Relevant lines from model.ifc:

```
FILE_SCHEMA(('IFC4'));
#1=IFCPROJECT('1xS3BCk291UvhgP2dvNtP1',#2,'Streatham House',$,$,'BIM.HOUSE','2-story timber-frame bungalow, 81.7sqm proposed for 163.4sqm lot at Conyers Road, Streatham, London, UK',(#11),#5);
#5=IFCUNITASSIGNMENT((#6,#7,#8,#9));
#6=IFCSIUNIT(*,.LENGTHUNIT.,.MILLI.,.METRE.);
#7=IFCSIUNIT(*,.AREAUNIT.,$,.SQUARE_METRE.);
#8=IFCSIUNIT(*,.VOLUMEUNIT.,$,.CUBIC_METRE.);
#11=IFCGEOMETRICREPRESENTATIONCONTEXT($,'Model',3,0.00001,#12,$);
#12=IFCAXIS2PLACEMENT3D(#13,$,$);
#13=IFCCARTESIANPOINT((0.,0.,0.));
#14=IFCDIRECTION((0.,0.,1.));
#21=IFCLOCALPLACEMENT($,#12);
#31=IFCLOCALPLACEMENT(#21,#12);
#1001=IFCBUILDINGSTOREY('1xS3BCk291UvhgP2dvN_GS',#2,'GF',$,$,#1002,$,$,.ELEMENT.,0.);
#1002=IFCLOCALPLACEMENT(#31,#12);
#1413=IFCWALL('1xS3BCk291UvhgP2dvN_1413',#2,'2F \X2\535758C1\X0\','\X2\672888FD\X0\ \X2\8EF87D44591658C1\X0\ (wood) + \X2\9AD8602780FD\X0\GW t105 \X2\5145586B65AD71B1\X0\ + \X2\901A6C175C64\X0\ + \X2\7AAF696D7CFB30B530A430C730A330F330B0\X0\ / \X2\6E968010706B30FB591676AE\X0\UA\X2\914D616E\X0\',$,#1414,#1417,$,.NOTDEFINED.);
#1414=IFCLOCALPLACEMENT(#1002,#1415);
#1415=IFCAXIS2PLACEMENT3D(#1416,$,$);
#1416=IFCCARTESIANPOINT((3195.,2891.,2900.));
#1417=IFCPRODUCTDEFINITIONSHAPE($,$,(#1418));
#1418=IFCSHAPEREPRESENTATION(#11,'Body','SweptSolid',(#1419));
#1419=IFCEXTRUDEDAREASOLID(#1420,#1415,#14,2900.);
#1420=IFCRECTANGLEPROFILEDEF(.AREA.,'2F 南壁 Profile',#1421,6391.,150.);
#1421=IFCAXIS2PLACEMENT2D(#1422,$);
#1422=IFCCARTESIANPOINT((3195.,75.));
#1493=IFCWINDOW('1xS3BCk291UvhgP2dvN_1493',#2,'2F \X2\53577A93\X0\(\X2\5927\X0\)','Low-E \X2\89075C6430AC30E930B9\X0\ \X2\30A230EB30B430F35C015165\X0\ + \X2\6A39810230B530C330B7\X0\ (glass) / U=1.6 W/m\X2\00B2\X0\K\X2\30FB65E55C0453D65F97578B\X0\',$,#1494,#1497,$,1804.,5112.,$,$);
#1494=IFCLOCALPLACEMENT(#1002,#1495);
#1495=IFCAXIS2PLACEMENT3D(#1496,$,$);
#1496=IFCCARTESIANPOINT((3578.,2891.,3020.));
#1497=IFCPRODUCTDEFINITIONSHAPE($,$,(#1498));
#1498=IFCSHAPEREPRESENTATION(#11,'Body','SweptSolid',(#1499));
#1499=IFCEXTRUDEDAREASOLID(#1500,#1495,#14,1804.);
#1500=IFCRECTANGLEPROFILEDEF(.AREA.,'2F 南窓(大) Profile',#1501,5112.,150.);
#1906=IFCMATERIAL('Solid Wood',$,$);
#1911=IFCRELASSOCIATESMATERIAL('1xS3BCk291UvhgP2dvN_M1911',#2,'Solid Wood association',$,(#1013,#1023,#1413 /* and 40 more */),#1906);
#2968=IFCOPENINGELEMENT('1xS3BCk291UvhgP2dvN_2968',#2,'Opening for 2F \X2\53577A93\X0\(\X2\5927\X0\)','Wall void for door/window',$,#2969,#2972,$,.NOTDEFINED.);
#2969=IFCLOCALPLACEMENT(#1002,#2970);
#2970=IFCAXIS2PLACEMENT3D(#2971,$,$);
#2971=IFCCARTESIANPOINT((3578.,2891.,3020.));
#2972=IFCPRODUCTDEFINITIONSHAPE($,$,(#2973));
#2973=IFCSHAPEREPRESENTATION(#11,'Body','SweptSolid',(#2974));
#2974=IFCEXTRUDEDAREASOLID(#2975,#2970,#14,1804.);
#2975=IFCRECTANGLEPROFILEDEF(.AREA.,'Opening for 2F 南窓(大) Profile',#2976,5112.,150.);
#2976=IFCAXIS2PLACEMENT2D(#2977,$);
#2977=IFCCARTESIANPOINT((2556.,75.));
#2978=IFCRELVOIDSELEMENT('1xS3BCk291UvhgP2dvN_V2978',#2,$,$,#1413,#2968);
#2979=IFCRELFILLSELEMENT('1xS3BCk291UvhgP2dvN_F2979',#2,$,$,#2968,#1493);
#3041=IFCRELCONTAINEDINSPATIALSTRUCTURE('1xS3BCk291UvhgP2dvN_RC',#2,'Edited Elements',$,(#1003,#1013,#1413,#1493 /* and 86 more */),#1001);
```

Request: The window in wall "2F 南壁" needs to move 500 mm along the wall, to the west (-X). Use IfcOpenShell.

```python
import ifcopenshell
import ifcopenshell.api.geometry
import ifcopenshell.util.placement
import ifcopenshell.util.unit

model = ifcopenshell.open("model.ifc")
unit_scale = ifcopenshell.util.unit.calculate_unit_scale(model)

window = model.by_guid("1xS3BCk291UvhgP2dvN_1493")
opening = window.FillsVoids[0].RelatingOpeningElement
wall = opening.VoidsElements[0].RelatingBuildingElement

wall_matrix = ifcopenshell.util.placement.get_local_placement(wall.ObjectPlacement)
shift = wall_matrix[:3, 0] * -0.5 / unit_scale
before = ifcopenshell.util.placement.get_local_placement(window.ObjectPlacement)[:3, 3].copy()

# The window is not placed relative to its opening, so move both.
for product in (opening, window):
    matrix = ifcopenshell.util.placement.get_local_placement(product.ObjectPlacement)
    matrix[:3, 3] += shift
    ifcopenshell.api.geometry.edit_object_placement(model, product=product, matrix=matrix, is_si=False)

after = ifcopenshell.util.placement.get_local_placement(window.ObjectPlacement)[:3, 3]
print("window moved by", (after - before).round(3) + 0.0)

model.write("model_rev.ifc")
```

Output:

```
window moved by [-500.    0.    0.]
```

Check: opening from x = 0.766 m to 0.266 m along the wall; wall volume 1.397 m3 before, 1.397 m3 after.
